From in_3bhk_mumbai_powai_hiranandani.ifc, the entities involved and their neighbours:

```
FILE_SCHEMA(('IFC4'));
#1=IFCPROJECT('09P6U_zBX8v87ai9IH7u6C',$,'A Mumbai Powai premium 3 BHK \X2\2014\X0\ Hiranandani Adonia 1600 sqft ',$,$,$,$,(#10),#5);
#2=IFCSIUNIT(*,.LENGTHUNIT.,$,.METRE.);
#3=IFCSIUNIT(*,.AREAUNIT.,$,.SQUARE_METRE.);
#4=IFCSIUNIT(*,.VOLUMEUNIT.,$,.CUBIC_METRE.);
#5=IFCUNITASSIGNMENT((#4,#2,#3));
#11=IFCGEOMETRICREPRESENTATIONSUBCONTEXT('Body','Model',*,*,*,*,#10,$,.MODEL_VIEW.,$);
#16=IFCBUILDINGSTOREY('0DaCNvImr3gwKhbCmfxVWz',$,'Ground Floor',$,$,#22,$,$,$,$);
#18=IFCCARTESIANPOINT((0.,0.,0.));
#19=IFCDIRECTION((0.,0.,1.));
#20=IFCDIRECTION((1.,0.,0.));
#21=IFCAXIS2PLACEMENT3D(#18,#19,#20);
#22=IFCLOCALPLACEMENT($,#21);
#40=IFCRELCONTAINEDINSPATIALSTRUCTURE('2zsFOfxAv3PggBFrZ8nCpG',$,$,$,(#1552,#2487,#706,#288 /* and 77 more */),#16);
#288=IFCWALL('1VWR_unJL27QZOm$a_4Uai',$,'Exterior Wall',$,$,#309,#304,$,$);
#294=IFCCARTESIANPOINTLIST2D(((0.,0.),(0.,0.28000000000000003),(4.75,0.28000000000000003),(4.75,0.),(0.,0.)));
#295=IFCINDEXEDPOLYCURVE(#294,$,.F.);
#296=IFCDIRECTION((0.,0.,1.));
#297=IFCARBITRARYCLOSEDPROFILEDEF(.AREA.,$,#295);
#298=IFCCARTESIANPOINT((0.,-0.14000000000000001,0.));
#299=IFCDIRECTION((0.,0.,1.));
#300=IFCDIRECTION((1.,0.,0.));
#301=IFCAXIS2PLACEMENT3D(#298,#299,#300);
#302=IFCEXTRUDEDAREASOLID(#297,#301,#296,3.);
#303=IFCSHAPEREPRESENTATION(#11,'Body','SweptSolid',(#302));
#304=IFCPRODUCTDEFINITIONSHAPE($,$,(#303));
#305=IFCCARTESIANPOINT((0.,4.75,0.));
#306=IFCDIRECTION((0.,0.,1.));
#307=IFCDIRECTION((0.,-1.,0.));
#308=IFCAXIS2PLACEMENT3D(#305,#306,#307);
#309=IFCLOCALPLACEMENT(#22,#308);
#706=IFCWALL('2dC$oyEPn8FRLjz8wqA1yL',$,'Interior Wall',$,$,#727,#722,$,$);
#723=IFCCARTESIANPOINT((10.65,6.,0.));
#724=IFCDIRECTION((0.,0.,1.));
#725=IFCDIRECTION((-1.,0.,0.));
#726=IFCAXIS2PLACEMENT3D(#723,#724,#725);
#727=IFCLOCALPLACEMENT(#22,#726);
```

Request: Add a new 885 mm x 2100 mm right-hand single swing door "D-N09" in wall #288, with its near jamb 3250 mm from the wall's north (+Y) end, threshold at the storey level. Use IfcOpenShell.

```python
import numpy as np
import ifcopenshell
import ifcopenshell.api.feature
import ifcopenshell.api.geometry
import ifcopenshell.api.root
import ifcopenshell.api.spatial
import ifcopenshell.geom
import ifcopenshell.util.element
import ifcopenshell.util.placement
import ifcopenshell.util.representation
import ifcopenshell.util.shape
import ifcopenshell.util.unit

model = ifcopenshell.open("in_3bhk_mumbai_powai_hiranandani.ifc")
unit_scale = ifcopenshell.util.unit.calculate_unit_scale(model)
settings = ifcopenshell.geom.settings()


def volume(element):
    """Net volume in cubic metres, openings subtracted."""
    shape = ifcopenshell.geom.create_shape(settings, element)
    return ifcopenshell.util.shape.get_volume(shape.geometry)


wall = model.by_id(288)
storey = ifcopenshell.util.element.get_container(wall, ifc_class="IfcBuildingStorey")
context = ifcopenshell.util.representation.get_context(model, "Model", "Body", "MODEL_VIEW")
before = volume(wall)

width, height, from_end, sill = 0.885, 2.1, 3.25, 0.0  # metres

# The wall runs along its own X axis, and the end named is its -X end.
wall_shape = ifcopenshell.geom.create_shape(settings, wall)
x, y, z = ifcopenshell.util.shape.get_vertices(wall_shape.geometry).T
start = x.min() + from_end
face, thickness = float(y.min()), float(y.max() - y.min())
wall_matrix = ifcopenshell.util.placement.get_local_placement(wall.ObjectPlacement)
level = ifcopenshell.util.placement.get_local_placement(storey.ObjectPlacement)[2, 3]


def in_wall(x, y):
    """Placement at x, y metres in the wall's axes, at sill height."""
    matrix = wall_matrix.copy()
    matrix[:, 3] = wall_matrix @ np.array([x / unit_scale, y / unit_scale, 0.0, 1.0])
    matrix[2, 3] = level + sill / unit_scale
    return matrix


# Opening: a box that overshoots both wall faces by 50 mm.
opening = ifcopenshell.api.root.create_entity(model, ifc_class="IfcOpeningElement", predefined_type="OPENING")
box = ifcopenshell.api.geometry.add_wall_representation(
    model, context=context, length=width, height=height, thickness=thickness + 0.1
)
ifcopenshell.api.geometry.assign_representation(model, product=opening, representation=box)
ifcopenshell.api.geometry.edit_object_placement(model, product=opening, matrix=in_wall(start, face - 0.05), is_si=False)
ifcopenshell.api.feature.add_feature(model, feature=opening, element=wall)

door = ifcopenshell.api.root.create_entity(model, ifc_class="IfcDoor", name="D-N09", predefined_type="DOOR")
door.OverallWidth, door.OverallHeight = width / unit_scale, height / unit_scale
door.OperationType = "SINGLE_SWING_RIGHT"
body = ifcopenshell.api.geometry.add_door_representation(
    model,
    context=context,
    overall_width=door.OverallWidth,
    overall_height=door.OverallHeight,
    operation_type="SINGLE_SWING_RIGHT",
    lining_properties={"LiningDepth": thickness / unit_scale, "ThresholdDepth": thickness / unit_scale},
)
ifcopenshell.api.geometry.assign_representation(model, product=door, representation=body)
ifcopenshell.api.spatial.assign_container(model, products=[door], relating_structure=storey)
ifcopenshell.api.feature.add_filling(model, opening=opening, element=door)

# The lining spans the wall, so the door starts at the wall face.
ifcopenshell.api.geometry.edit_object_placement(model, product=door, matrix=in_wall(start, face), is_si=False)

after = volume(wall)

print(f"wall volume {before:.3f} -> {after:.3f} m3")

model.write("in_3bhk_mumbai_powai_hiranandani_v2.ifc")
```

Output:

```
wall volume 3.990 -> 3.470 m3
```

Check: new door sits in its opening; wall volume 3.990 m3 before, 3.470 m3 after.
